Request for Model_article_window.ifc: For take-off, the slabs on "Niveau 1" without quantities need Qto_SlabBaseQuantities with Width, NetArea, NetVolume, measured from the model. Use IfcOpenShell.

First a look at what the model holds.

```python
import ifcopenshell
import ifcopenshell.util.element
import ifcopenshell.util.unit

model = ifcopenshell.open("Model_article_window.ifc")
print(model.schema)
for unit_type in ("LENGTHUNIT", "AREAUNIT", "VOLUMEUNIT"):
    print(unit_type, ifcopenshell.util.unit.calculate_unit_scale(model, unit_type))
storey = next(s for s in model.by_type("IfcBuildingStorey") if s.Name == "Niveau 1")
slabs = [e for e in ifcopenshell.util.element.get_decomposition(storey) if e.is_a("IfcSlab")]
for e in sorted(slabs, key=lambda e: e.id()):
    print(e.id(), e.is_a(), e.Name, list(ifcopenshell.util.element.get_psets(e, qtos_only=True)), sep=" | ")
```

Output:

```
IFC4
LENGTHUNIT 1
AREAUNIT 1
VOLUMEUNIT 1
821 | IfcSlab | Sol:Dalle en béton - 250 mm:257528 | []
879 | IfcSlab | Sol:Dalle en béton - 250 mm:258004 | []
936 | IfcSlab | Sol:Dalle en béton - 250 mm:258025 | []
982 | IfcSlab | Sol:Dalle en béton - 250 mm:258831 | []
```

```python
import ifcopenshell
import ifcopenshell.api.pset
import ifcopenshell.geom
import ifcopenshell.util.element
import ifcopenshell.util.shape
import ifcopenshell.util.unit

model = ifcopenshell.open("Model_article_window.ifc")
unit_scale = ifcopenshell.util.unit.calculate_unit_scale(model)
area_scale = ifcopenshell.util.unit.calculate_unit_scale(model, "AREAUNIT")
volume_scale = ifcopenshell.util.unit.calculate_unit_scale(model, "VOLUMEUNIT")
settings = ifcopenshell.geom.settings()

storey = next(s for s in model.by_type("IfcBuildingStorey") if s.Name == "Niveau 1")
slabs = [e for e in ifcopenshell.util.element.get_decomposition(storey) if e.is_a("IfcSlab")]

for e in sorted(slabs, key=lambda e: e.id()):
    if ifcopenshell.util.element.get_psets(e, qtos_only=True, should_inherit=False):
        continue
    # Geometry comes back in metres, in the element's own axes.
    shape = ifcopenshell.geom.create_shape(settings, e)
    values = {
        "Width": ifcopenshell.util.shape.get_z(shape.geometry) / unit_scale,
        "NetArea": ifcopenshell.util.shape.get_footprint_area(shape.geometry) / area_scale,
        "NetVolume": ifcopenshell.util.shape.get_volume(shape.geometry) / volume_scale,
    }
    qto = ifcopenshell.api.pset.add_qto(model, product=e, name="Qto_SlabBaseQuantities")
    ifcopenshell.api.pset.edit_qto(model, qto=qto, properties=values)
    print(e.id(), {k: round(v, 3) for k, v in values.items()})

model.write("Model_article_window-out.ifc")
```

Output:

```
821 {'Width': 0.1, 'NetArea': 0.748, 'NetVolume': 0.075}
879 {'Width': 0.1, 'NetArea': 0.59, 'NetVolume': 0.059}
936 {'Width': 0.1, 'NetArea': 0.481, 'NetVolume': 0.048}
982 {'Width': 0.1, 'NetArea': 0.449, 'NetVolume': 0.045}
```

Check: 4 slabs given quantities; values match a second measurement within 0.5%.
